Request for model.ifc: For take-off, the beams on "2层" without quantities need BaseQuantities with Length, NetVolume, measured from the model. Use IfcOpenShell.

First a look at what the model holds.

```python
import ifcopenshell
import ifcopenshell.util.element
import ifcopenshell.util.unit

model = ifcopenshell.open("model.ifc")
print(model.schema)
for unit_type in ("LENGTHUNIT", "AREAUNIT", "VOLUMEUNIT"):
    print(unit_type, ifcopenshell.util.unit.calculate_unit_scale(model, unit_type))
storey = next(s for s in model.by_type("IfcBuildingStorey") if s.Name == "2层")
beams = [e for e in ifcopenshell.util.element.get_decomposition(storey) if e.is_a("IfcBeam")]
for e in sorted(beams, key=lambda e: e.id()):
    print(e.id(), e.is_a(), e.Name, list(ifcopenshell.util.element.get_psets(e, qtos_only=True)), sep=" | ")
```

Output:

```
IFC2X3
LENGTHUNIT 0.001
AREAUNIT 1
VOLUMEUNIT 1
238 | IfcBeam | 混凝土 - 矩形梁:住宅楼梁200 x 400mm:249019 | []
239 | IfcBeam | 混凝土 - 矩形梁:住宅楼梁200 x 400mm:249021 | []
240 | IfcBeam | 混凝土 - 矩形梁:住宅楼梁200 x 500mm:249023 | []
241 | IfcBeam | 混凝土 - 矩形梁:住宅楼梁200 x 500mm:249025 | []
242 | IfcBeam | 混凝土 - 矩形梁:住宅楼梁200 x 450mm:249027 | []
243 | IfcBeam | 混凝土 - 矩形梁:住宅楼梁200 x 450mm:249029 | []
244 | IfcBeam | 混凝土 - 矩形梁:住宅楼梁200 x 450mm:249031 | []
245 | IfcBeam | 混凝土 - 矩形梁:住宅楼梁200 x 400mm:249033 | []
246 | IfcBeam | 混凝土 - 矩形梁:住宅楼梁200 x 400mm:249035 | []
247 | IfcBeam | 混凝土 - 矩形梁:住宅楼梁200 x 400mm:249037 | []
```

```python
import ifcopenshell
import ifcopenshell.api.pset
import ifcopenshell.geom
import ifcopenshell.util.element
import ifcopenshell.util.shape
import ifcopenshell.util.unit

model = ifcopenshell.open("model.ifc")
unit_scale = ifcopenshell.util.unit.calculate_unit_scale(model)
volume_scale = ifcopenshell.util.unit.calculate_unit_scale(model, "VOLUMEUNIT")
settings = ifcopenshell.geom.settings()

storey = next(s for s in model.by_type("IfcBuildingStorey") if s.Name == "2层")
beams = [e for e in ifcopenshell.util.element.get_decomposition(storey) if e.is_a("IfcBeam")]

for e in sorted(beams, key=lambda e: e.id()):
    if ifcopenshell.util.element.get_psets(e, qtos_only=True, should_inherit=False):
        continue
    # Geometry comes back in metres, in the element's own axes.
    shape = ifcopenshell.geom.create_shape(settings, e)
    values = {
        "Length": ifcopenshell.util.shape.get_max_xyz(shape.geometry) / unit_scale,
        "NetVolume": ifcopenshell.util.shape.get_volume(shape.geometry) / volume_scale,
    }
    qto = ifcopenshell.api.pset.add_qto(model, product=e, name="BaseQuantities")
    ifcopenshell.api.pset.edit_qto(model, qto=qto, properties=values)
    print(e.id(), {k: round(v, 3) for k, v in values.items()})

model.write("model_rev.ifc")
```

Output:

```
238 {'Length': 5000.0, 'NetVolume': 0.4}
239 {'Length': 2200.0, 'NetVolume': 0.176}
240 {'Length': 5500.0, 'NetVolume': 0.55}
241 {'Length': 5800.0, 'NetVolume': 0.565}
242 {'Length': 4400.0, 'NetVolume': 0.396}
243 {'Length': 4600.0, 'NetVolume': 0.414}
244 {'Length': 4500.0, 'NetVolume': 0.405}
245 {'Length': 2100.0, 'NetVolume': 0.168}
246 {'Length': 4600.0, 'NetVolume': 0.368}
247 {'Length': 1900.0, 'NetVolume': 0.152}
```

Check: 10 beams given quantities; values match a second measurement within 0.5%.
